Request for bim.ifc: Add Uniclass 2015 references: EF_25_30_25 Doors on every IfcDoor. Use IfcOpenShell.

First a look at what the model holds.

```python
import ifcopenshell

model = ifcopenshell.open("bim.ifc")
print(model.schema)
print("classifications:", [c.Name for c in model.by_type("IfcClassification")])
for ifc_class in ("IfcDoor", "IfcRoof", "IfcStair", "IfcWall", "IfcWindow"):
    print(ifc_class, len(model.by_type(ifc_class)))
```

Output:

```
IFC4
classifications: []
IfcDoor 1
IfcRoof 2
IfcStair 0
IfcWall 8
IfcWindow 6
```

```python
import ifcopenshell
import ifcopenshell.api.classification

model = ifcopenshell.open("bim.ifc")

system = ifcopenshell.api.classification.add_classification(model, classification="Uniclass 2015")

codes = {
    "IfcDoor": ("EF_25_30_25", "Doors"),
}
for ifc_class, (code, name) in codes.items():
    products = model.by_type(ifc_class)
    ifcopenshell.api.classification.add_reference(
        model, products=products, classification=system, identification=code, name=name
    )
    print(code, len(products))

model.write("bim_updated.ifc")
```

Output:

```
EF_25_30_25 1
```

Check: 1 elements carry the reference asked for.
